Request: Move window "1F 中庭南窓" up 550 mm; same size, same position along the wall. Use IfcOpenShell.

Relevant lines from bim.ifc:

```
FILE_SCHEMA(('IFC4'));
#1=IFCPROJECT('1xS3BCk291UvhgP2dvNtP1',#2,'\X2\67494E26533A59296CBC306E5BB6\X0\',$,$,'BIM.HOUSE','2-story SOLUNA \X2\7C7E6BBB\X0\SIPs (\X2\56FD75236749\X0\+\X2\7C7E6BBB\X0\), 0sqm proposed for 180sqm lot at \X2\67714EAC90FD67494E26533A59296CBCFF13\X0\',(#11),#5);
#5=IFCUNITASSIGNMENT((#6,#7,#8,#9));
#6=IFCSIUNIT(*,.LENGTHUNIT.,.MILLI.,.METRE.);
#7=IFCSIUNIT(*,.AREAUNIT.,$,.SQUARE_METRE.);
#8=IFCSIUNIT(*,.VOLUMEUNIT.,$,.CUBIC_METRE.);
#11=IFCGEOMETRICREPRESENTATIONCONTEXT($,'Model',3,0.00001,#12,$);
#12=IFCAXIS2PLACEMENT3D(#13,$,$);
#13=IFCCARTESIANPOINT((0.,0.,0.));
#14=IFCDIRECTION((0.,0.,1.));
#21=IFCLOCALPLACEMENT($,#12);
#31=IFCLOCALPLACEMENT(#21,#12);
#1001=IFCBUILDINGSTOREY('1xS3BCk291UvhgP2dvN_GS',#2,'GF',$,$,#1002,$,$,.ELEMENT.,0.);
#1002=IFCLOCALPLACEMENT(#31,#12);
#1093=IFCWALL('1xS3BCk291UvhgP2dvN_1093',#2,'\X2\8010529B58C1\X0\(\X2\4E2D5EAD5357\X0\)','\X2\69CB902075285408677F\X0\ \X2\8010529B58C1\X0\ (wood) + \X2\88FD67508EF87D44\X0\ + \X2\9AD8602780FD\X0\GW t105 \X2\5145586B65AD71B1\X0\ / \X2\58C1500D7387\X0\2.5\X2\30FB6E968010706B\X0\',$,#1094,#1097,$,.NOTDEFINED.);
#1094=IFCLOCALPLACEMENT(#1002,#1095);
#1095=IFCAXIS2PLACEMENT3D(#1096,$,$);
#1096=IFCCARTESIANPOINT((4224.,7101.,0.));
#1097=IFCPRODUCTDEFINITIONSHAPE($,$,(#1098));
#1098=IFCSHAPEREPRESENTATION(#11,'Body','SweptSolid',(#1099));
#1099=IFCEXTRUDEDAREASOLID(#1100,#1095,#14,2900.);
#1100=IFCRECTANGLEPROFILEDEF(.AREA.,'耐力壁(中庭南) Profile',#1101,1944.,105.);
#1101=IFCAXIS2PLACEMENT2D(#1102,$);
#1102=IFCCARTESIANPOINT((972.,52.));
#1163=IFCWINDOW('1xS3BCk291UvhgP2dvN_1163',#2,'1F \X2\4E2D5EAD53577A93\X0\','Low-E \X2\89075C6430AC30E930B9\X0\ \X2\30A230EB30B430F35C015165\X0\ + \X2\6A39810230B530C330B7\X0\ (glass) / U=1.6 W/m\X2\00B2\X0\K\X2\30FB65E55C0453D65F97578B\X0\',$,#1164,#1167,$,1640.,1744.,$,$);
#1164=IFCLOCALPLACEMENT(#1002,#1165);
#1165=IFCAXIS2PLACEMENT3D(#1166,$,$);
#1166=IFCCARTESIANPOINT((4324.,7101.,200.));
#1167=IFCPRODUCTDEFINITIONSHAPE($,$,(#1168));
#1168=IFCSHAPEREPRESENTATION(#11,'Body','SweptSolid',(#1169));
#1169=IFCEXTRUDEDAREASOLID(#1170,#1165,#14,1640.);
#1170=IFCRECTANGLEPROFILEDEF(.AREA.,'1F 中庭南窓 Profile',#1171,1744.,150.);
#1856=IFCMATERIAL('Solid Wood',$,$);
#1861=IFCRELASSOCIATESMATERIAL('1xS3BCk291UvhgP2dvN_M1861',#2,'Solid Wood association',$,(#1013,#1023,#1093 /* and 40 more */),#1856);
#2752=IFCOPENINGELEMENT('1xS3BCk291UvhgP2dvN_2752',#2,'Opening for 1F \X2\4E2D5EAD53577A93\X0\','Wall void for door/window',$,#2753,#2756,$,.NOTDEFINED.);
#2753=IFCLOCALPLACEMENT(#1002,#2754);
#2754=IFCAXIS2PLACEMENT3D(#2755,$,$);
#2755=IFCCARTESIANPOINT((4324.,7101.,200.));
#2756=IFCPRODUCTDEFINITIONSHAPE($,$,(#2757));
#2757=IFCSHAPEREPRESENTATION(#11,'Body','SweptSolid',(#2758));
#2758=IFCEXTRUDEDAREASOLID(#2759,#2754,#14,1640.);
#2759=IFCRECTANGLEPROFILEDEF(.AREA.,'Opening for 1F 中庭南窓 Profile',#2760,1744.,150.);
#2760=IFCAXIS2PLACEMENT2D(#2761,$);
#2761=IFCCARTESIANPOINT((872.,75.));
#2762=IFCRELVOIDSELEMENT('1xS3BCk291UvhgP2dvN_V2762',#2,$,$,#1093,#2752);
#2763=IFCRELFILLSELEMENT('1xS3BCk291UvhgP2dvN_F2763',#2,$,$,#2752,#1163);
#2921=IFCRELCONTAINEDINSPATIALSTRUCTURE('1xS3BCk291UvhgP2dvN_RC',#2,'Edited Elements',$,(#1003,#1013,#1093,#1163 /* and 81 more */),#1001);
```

```python
import numpy as np
import ifcopenshell
import ifcopenshell.api.geometry
import ifcopenshell.util.placement
import ifcopenshell.util.unit

model = ifcopenshell.open("bim.ifc")
unit_scale = ifcopenshell.util.unit.calculate_unit_scale(model)

window = model.by_guid("1xS3BCk291UvhgP2dvN_1163")
opening = window.FillsVoids[0].RelatingOpeningElement
dz = 0.55 / unit_scale

shift = np.array([0.0, 0.0, dz])
# The window is not placed relative to its opening, so move both.
for product in (opening, window):
    matrix = ifcopenshell.util.placement.get_local_placement(product.ObjectPlacement)
    matrix[:3, 3] += shift
    ifcopenshell.api.geometry.edit_object_placement(model, product=product, matrix=matrix, is_si=False)

print(f"moved by {dz * unit_scale:+.3f} m")

model.write("bim-out.ifc")
```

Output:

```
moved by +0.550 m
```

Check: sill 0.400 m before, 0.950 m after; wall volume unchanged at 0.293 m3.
